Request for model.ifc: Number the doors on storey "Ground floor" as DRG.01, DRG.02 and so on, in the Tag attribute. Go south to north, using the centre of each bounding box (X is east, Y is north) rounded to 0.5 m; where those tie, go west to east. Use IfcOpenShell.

First a look at what the model holds.

```python
import ifcopenshell
import ifcopenshell.util.element
import ifcopenshell.util.placement

model = ifcopenshell.open("model.ifc")
print(model.schema)
storey = next(s for s in model.by_type("IfcBuildingStorey") if s.Name == "Ground floor")
doors = [e for e in ifcopenshell.util.element.get_decomposition(storey) if e.is_a("IfcDoor")]
for e in sorted(doors, key=lambda e: e.id()):
    origin = ifcopenshell.util.placement.get_local_placement(e.ObjectPlacement)[:3, 3]
    print(e.id(), e.Tag, e.Name, origin.round(2) + 0.0, sep=" | ")
```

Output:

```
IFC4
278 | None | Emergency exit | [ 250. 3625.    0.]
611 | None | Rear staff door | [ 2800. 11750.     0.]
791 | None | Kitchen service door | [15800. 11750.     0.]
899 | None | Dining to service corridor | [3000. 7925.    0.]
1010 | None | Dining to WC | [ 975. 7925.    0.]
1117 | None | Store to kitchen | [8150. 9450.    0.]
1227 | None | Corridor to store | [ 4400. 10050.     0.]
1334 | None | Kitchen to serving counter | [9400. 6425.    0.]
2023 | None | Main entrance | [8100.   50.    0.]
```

```python
import ifcopenshell
import ifcopenshell.geom
import ifcopenshell.util.element
import ifcopenshell.util.shape

model = ifcopenshell.open("model.ifc")
settings = ifcopenshell.geom.settings()
settings.set("use-world-coords", True)


def centre(element):
    shape = ifcopenshell.geom.create_shape(settings, element)
    return ifcopenshell.util.shape.get_bbox_centroid(shape.geometry)


storey = next(s for s in model.by_type("IfcBuildingStorey") if s.Name == "Ground floor")
doors = [e for e in ifcopenshell.util.element.get_decomposition(storey) if e.is_a("IfcDoor")]

# Insertion points can sit at a corner or the storey origin, so sort by the geometry (in metres).
centres = {e: centre(e) for e in doors}
doors.sort(key=lambda e: (round(centres[e][1] / 0.5), centres[e][0]))

for i, e in enumerate(doors, start=1):
    number = f"DRG.{i:02d}"
    e.Tag = number
    print(e.id(), number)

model.write("model_edited.ifc")
```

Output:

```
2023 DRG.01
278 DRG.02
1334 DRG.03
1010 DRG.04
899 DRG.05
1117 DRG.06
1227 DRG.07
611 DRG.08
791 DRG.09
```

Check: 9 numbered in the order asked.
